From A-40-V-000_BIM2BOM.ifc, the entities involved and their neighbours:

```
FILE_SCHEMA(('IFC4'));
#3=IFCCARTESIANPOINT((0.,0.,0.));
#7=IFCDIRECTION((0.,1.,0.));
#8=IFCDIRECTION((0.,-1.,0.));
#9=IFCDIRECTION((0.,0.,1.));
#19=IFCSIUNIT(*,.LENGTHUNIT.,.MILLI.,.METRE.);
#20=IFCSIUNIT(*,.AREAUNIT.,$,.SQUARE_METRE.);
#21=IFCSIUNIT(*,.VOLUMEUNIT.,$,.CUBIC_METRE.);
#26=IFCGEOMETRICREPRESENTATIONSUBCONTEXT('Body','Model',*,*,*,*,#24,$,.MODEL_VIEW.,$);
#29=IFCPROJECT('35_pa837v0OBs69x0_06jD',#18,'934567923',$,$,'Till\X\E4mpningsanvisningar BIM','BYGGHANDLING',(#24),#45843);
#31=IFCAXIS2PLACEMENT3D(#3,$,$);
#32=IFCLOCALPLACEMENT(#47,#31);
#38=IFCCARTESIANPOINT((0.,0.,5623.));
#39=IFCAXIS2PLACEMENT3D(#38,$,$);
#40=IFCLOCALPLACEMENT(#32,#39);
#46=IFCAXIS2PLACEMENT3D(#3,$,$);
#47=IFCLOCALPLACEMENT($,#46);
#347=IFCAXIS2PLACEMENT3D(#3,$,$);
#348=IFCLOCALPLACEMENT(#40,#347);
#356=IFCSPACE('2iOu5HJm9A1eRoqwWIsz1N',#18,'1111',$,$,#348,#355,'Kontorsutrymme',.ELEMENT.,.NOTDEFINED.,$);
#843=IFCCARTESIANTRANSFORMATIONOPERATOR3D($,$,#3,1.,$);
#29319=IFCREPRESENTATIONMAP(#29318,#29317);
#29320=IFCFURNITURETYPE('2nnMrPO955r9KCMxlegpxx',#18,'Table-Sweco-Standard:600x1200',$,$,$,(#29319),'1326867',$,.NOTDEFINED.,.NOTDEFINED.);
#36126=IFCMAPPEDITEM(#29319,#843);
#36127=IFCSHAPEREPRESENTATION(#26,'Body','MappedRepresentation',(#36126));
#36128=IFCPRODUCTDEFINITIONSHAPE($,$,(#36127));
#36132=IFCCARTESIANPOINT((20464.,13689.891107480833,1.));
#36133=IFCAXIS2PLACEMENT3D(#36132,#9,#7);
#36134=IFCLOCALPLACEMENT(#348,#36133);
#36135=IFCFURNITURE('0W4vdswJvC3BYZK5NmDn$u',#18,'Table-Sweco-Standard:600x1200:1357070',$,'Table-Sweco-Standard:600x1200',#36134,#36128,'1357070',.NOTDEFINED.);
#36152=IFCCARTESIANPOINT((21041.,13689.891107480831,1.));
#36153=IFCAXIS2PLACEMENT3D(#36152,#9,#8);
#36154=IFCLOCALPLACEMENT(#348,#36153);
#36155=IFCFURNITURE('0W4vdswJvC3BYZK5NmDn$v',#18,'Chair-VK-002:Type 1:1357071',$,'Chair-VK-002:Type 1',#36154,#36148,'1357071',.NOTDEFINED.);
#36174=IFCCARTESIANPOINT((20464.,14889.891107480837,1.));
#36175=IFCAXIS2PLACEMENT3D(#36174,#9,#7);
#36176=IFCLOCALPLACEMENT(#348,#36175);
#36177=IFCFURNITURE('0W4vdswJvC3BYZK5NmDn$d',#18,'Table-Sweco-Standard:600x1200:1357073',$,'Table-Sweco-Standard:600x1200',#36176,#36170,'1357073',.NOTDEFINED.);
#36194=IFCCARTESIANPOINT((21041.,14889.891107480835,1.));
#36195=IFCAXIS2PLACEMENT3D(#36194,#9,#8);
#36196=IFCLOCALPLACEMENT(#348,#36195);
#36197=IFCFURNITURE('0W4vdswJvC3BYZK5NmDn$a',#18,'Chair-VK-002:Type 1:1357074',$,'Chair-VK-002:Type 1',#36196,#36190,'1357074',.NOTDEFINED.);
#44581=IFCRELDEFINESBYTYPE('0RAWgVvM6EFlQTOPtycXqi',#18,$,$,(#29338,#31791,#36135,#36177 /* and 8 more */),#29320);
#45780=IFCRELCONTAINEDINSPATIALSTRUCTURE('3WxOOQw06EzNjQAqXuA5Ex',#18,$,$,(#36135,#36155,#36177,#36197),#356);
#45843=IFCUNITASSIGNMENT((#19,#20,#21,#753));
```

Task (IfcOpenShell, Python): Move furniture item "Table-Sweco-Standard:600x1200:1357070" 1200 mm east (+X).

```python
import ifcopenshell
import ifcopenshell.api.geometry
import ifcopenshell.util.placement

model = ifcopenshell.open("A-40-V-000_BIM2BOM.ifc")

item = model.by_guid("0W4vdswJvC3BYZK5NmDn$u")
matrix = ifcopenshell.util.placement.get_local_placement(item.ObjectPlacement)
matrix[0, 3] += 1200.0
ifcopenshell.api.geometry.edit_object_placement(model, product=item, matrix=matrix, is_si=False)

print(ifcopenshell.util.placement.get_local_placement(item.ObjectPlacement).round(3) + 0.0)

model.write("A-40-V-000_BIM2BOM_v2.ifc")
```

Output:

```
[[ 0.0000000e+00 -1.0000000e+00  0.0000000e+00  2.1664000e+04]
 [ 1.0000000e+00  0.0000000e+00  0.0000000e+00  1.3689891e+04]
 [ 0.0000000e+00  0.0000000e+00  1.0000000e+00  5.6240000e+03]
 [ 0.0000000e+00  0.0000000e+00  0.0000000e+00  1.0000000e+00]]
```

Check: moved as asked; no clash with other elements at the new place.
